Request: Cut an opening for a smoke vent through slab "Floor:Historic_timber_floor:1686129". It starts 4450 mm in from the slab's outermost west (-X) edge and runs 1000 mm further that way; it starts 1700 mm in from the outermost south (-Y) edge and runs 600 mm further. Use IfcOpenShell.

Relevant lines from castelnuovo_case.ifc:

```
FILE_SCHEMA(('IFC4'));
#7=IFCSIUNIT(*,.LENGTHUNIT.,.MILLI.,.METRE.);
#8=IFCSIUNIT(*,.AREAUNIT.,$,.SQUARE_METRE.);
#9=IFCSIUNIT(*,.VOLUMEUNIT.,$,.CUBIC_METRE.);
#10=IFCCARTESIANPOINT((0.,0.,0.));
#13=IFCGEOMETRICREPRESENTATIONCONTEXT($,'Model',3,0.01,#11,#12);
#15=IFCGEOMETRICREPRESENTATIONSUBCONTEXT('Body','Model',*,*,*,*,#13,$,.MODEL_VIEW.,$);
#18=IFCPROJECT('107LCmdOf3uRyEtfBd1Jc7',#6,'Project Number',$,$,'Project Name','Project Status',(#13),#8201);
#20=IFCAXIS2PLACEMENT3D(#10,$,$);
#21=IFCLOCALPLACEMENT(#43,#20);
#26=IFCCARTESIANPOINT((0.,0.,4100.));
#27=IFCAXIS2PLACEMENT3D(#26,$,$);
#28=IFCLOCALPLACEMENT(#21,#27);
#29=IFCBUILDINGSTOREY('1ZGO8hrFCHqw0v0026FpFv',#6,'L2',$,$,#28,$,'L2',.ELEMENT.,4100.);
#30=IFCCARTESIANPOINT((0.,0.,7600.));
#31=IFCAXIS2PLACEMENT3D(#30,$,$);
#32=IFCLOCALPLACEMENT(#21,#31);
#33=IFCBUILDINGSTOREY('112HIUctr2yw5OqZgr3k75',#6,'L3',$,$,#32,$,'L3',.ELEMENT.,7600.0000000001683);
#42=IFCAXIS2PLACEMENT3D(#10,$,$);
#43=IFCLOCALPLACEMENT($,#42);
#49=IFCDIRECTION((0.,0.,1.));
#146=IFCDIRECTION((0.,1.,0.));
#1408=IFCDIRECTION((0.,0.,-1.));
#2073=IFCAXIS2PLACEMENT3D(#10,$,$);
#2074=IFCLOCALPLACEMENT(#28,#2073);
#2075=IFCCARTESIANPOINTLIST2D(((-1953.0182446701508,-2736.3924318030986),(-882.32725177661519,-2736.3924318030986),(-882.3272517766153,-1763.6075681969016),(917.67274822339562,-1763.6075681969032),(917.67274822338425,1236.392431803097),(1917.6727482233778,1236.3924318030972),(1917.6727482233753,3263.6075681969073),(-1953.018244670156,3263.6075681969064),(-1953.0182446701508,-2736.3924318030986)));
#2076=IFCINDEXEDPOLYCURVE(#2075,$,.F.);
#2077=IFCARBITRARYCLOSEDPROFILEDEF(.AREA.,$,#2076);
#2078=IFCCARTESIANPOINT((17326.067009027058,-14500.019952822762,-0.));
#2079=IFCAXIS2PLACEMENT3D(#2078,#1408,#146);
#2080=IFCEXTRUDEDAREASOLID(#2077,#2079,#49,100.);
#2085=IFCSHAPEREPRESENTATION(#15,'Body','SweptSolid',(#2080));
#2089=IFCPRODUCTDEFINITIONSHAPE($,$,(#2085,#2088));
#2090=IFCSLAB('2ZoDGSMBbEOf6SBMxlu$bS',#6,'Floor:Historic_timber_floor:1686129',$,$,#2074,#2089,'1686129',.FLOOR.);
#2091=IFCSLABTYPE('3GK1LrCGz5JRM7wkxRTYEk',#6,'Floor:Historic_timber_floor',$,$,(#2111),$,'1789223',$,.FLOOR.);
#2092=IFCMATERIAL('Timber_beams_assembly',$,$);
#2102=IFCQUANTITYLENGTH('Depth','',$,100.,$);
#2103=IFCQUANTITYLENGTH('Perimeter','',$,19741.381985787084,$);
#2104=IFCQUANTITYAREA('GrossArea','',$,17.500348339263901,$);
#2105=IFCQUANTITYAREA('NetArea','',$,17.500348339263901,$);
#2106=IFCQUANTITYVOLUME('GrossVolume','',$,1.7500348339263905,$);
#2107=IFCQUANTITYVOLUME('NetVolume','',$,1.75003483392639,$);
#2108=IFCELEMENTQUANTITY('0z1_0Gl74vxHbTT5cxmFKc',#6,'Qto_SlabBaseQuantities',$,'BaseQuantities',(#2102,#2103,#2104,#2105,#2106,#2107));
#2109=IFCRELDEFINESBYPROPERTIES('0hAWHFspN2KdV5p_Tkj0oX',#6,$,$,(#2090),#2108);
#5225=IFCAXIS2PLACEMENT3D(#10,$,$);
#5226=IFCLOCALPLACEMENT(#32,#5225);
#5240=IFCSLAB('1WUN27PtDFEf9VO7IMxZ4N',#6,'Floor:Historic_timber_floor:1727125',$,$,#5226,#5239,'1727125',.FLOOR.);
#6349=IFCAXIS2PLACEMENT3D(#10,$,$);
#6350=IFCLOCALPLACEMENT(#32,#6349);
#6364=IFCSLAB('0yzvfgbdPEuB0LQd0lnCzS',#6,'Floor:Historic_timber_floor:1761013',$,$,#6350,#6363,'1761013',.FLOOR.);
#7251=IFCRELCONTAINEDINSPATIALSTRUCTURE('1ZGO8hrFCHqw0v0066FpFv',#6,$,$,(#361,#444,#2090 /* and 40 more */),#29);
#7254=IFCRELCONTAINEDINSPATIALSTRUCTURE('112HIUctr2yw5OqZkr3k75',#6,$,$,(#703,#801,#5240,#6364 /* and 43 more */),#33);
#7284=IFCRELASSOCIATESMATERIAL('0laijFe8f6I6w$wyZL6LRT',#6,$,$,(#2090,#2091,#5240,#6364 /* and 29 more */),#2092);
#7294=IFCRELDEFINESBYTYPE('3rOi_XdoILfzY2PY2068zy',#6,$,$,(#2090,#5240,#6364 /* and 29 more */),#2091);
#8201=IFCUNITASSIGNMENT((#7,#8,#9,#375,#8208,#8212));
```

```python
import numpy as np
import ifcopenshell
import ifcopenshell.api.feature
import ifcopenshell.api.geometry
import ifcopenshell.api.pset
import ifcopenshell.api.root
import ifcopenshell.geom
import ifcopenshell.util.element
import ifcopenshell.util.placement
import ifcopenshell.util.representation
import ifcopenshell.util.shape
import ifcopenshell.util.unit

model = ifcopenshell.open("castelnuovo_case.ifc")
unit_scale = ifcopenshell.util.unit.calculate_unit_scale(model)
area_scale = ifcopenshell.util.unit.calculate_unit_scale(model, "AREAUNIT")
volume_scale = ifcopenshell.util.unit.calculate_unit_scale(model, "VOLUMEUNIT")
settings = ifcopenshell.geom.settings()


def volume(element):
    """Net volume in cubic metres, openings subtracted."""
    shape = ifcopenshell.geom.create_shape(settings, element)
    return ifcopenshell.util.shape.get_volume(shape.geometry)


slab = model.by_guid("2ZoDGSMBbEOf6SBMxlu$bS")
before = volume(slab)

# Extent in the slab's own axes, in metres. The edges named are its -X and -Y sides.
slab_shape = ifcopenshell.geom.create_shape(settings, slab)
vertices = ifcopenshell.util.shape.get_vertices(slab_shape.geometry)
x_min, y_min, bottom = vertices.min(axis=0)
top = vertices[:, 2].max()

opening = ifcopenshell.api.root.create_entity(model, ifc_class="IfcOpeningElement", name="Smoke vent opening", predefined_type="OPENING")
context = ifcopenshell.util.representation.get_context(model, "Model", "Body", "MODEL_VIEW")
width, depth = 1, 0.6
outline = [(0.0, 0.0), (width, 0.0), (width, depth), (0.0, depth), (0.0, 0.0)]
# Overshoot both faces by 50 mm so the cut is clean.
shape = ifcopenshell.api.geometry.add_slab_representation(
    model, context=context, depth=top - bottom + 0.1, polyline=outline
)
ifcopenshell.api.geometry.assign_representation(model, product=opening, representation=shape)

matrix = ifcopenshell.util.placement.get_local_placement(slab.ObjectPlacement)
matrix[:, 3] = matrix @ np.append(np.array([x_min + 4.45, y_min + 1.7, bottom - 0.05]) / unit_scale, 1.0)
ifcopenshell.api.geometry.edit_object_placement(model, product=opening, matrix=matrix, is_si=False)
ifcopenshell.api.feature.add_feature(model, feature=opening, element=slab)

after = volume(slab)

# Update the slab's stored quantities.
qto = model.by_id(ifcopenshell.util.element.get_pset(slab, "Qto_SlabBaseQuantities", should_inherit=False)["id"])
ifcopenshell.api.pset.edit_qto(model, qto=qto, properties={
    "NetArea": after / (top - bottom) / area_scale,
    "NetVolume": after / volume_scale,
})

print(f"slab volume {before:.3f} -> {after:.3f} m3")

model.write("castelnuovo_case_updated.ifc")
```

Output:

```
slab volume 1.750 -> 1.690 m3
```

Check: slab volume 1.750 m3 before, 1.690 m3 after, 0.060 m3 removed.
